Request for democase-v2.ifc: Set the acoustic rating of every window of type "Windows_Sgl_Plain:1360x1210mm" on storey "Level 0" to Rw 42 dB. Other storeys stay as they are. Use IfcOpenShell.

First a look at what the model holds.

```python
import ifcopenshell
import ifcopenshell.util.element

model = ifcopenshell.open("democase-v2.ifc")
print(model.schema)
storey = next(s for s in model.by_type("IfcBuildingStorey") if s.Name == "Level 0")
windows = [e for e in ifcopenshell.util.element.get_decomposition(storey) if e.is_a("IfcWindow")]
seen = {}
for e in windows:
    element_type = ifcopenshell.util.element.get_type(e)
    key = (element_type.Name if element_type != e and element_type else None, ifcopenshell.util.element.get_pset(e, "Pset_WindowCommon", "AcousticRating"))
    seen[key] = seen.get(key, 0) + 1
for (name, value), count in sorted(seen.items(), key=str):
    print(count, "x", name, "|", value)
```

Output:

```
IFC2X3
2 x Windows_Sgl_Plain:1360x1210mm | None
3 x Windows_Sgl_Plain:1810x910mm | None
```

```python
import ifcopenshell
import ifcopenshell.api.pset
import ifcopenshell.util.element

model = ifcopenshell.open("democase-v2.ifc")

storey = next(s for s in model.by_type("IfcBuildingStorey") if s.Name == "Level 0")
windows = [e for e in ifcopenshell.util.element.get_decomposition(storey) if e.is_a("IfcWindow")]

count = 0
for e in windows:
    element_type = ifcopenshell.util.element.get_type(e)
    if element_type in (None, e) or element_type.Name != "Windows_Sgl_Plain:1360x1210mm":
        continue
    # add_pset returns the element's existing set when there is one.
    pset = ifcopenshell.api.pset.add_pset(model, product=e, name="Pset_WindowCommon")
    ifcopenshell.api.pset.edit_pset(model, pset=pset, properties={"AcousticRating": "Rw 42 dB"})
    count += 1

print(count, "windows updated")

model.write("democase-v2-out.ifc")
```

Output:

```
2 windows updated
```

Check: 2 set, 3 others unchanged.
